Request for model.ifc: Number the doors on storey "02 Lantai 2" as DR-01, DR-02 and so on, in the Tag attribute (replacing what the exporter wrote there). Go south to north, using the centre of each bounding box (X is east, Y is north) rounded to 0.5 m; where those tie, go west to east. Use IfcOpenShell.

First a look at what the model holds.

```python
import ifcopenshell
import ifcopenshell.util.element
import ifcopenshell.util.placement

model = ifcopenshell.open("model.ifc")
print(model.schema)
storey = next(s for s in model.by_type("IfcBuildingStorey") if s.Name == "02 Lantai 2")
doors = [e for e in ifcopenshell.util.element.get_decomposition(storey) if e.is_a("IfcDoor")]
for e in sorted(doors, key=lambda e: e.id()):
    origin = ifcopenshell.util.placement.get_local_placement(e.ObjectPlacement)[:3, 3]
    print(e.id(), e.Tag, e.Name, origin.round(2) + 0.0, sep=" | ")
```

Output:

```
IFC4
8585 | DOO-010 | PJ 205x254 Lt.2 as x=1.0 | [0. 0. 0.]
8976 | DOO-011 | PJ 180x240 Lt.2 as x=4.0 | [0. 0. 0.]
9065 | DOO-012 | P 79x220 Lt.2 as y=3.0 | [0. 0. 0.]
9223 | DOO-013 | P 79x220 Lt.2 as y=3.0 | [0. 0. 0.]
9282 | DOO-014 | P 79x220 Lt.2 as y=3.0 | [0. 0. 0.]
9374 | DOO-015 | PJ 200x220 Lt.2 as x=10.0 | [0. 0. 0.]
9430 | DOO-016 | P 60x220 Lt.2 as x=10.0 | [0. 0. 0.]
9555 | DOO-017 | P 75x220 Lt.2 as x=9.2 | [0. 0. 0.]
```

```python
import ifcopenshell
import ifcopenshell.geom
import ifcopenshell.util.element
import ifcopenshell.util.shape

model = ifcopenshell.open("model.ifc")
settings = ifcopenshell.geom.settings()
settings.set("use-world-coords", True)


def centre(element):
    shape = ifcopenshell.geom.create_shape(settings, element)
    return ifcopenshell.util.shape.get_bbox_centroid(shape.geometry)


storey = next(s for s in model.by_type("IfcBuildingStorey") if s.Name == "02 Lantai 2")
doors = [e for e in ifcopenshell.util.element.get_decomposition(storey) if e.is_a("IfcDoor")]

# Insertion points can sit at a corner or the storey origin, so sort by the geometry (in metres).
centres = {e: centre(e) for e in doors}
doors.sort(key=lambda e: (round(centres[e][1] / 0.5), centres[e][0]))

for i, e in enumerate(doors, start=1):
    number = f"DR-{i:02d}"
    e.Tag = number
    print(e.id(), number)

model.write("model-out.ifc")
```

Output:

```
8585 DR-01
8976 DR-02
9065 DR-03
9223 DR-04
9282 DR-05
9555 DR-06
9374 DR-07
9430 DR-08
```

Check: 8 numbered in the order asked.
